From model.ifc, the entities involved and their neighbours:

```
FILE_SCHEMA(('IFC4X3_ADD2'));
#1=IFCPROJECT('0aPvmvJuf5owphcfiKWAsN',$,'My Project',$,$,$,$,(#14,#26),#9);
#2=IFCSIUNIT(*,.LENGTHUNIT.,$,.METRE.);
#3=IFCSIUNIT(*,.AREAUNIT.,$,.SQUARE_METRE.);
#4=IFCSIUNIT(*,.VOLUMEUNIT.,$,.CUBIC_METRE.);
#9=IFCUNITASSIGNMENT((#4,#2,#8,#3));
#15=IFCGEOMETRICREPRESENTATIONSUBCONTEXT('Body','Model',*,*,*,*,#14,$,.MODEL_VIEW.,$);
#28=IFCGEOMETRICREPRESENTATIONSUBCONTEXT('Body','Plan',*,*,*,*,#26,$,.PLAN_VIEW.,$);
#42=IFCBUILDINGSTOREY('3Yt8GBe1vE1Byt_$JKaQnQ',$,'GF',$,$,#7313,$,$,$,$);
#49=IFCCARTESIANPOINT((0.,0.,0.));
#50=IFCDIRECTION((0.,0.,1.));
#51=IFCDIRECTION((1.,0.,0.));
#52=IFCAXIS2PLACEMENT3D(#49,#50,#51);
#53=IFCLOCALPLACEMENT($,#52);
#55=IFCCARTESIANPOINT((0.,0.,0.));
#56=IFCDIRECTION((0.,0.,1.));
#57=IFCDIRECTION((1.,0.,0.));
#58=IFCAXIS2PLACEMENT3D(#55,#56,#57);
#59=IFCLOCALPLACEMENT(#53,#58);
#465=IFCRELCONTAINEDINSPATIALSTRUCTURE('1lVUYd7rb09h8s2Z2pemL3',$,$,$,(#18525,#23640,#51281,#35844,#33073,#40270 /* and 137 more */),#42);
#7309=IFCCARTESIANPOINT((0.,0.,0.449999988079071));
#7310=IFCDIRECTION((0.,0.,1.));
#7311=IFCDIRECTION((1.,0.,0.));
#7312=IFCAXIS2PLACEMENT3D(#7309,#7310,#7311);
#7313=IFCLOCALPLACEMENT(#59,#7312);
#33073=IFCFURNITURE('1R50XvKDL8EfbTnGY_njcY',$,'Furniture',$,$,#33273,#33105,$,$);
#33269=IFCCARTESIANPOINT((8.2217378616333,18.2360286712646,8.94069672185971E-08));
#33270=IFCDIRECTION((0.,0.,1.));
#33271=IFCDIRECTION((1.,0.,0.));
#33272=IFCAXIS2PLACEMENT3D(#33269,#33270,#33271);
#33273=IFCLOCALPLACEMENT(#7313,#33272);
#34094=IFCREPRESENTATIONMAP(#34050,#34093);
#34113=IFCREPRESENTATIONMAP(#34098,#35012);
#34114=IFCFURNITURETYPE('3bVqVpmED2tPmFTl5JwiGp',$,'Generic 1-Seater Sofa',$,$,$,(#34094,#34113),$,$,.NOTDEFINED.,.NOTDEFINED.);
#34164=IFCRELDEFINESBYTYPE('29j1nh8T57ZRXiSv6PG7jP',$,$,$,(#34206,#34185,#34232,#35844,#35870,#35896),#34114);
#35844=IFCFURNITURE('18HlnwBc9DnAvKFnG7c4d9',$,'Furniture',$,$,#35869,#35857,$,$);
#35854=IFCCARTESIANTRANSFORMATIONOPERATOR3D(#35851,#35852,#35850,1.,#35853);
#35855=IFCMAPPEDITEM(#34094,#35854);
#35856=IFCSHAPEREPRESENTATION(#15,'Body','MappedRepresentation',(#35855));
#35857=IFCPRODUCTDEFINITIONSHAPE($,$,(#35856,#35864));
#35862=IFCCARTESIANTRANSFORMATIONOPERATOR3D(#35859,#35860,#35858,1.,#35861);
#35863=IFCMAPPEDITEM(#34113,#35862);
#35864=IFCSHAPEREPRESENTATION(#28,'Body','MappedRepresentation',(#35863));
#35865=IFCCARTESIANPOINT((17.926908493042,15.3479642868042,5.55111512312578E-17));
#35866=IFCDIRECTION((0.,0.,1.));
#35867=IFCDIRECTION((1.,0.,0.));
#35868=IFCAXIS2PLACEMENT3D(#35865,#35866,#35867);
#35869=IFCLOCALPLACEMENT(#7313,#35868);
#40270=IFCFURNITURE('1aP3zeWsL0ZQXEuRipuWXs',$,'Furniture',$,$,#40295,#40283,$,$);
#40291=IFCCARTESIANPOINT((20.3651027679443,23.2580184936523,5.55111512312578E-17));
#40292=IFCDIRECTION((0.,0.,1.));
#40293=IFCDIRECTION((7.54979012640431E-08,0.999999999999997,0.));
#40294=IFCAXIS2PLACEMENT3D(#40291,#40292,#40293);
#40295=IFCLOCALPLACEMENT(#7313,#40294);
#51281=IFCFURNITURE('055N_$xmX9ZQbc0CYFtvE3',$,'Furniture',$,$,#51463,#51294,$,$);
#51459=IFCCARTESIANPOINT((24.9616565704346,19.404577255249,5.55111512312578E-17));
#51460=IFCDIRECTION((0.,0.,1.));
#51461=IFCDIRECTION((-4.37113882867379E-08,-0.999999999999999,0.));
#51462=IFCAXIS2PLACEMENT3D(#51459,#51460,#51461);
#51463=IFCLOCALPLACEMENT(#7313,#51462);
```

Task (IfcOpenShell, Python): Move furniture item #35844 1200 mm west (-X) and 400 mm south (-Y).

```python
import ifcopenshell
import ifcopenshell.api.geometry
import ifcopenshell.util.placement

model = ifcopenshell.open("model.ifc")

item = model.by_guid("18HlnwBc9DnAvKFnG7c4d9")
matrix = ifcopenshell.util.placement.get_local_placement(item.ObjectPlacement)
matrix[0, 3] -= 1.2
matrix[1, 3] -= 0.4
ifcopenshell.api.geometry.edit_object_placement(model, product=item, matrix=matrix, is_si=False)

print(ifcopenshell.util.placement.get_local_placement(item.ObjectPlacement).round(3) + 0.0)

model.write("model_v2.ifc")
```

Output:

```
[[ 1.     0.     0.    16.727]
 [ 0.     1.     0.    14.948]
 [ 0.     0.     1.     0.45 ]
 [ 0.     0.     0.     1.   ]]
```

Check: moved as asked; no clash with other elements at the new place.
